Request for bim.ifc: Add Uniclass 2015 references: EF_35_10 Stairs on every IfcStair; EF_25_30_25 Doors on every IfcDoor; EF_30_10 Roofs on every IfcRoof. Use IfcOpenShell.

First a look at what the model holds.

```python
import ifcopenshell

model = ifcopenshell.open("bim.ifc")
print(model.schema)
print("classifications:", [c.Name for c in model.by_type("IfcClassification")])
for ifc_class in ("IfcDoor", "IfcRoof", "IfcStair", "IfcWall", "IfcWindow"):
    print(ifc_class, len(model.by_type(ifc_class)))
```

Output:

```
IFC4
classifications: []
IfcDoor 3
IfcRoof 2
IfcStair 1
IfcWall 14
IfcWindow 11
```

```python
import ifcopenshell
import ifcopenshell.api.classification

model = ifcopenshell.open("bim.ifc")

system = ifcopenshell.api.classification.add_classification(model, classification="Uniclass 2015")

codes = {
    "IfcStair": ("EF_35_10", "Stairs"),
    "IfcDoor": ("EF_25_30_25", "Doors"),
    "IfcRoof": ("EF_30_10", "Roofs"),
}
for ifc_class, (code, name) in codes.items():
    products = model.by_type(ifc_class)
    ifcopenshell.api.classification.add_reference(
        model, products=products, classification=system, identification=code, name=name
    )
    print(code, len(products))

model.write("bim_v2.ifc")
```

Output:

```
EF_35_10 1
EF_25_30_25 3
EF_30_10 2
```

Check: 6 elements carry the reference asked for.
